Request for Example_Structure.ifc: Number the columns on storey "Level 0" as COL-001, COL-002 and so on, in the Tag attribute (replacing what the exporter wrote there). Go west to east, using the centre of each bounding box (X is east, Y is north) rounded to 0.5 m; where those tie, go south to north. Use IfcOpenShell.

First a look at what the model holds.

```python
import ifcopenshell
import ifcopenshell.util.element
import ifcopenshell.util.placement

model = ifcopenshell.open("Example_Structure.ifc")
print(model.schema)
storey = next(s for s in model.by_type("IfcBuildingStorey") if s.Name == "Level 0")
columns = [e for e in ifcopenshell.util.element.get_decomposition(storey) if e.is_a("IfcColumn")]
for e in sorted(columns, key=lambda e: e.id()):
    origin = ifcopenshell.util.placement.get_local_placement(e.ObjectPlacement)[:3, 3]
    print(e.id(), e.Tag, e.Name, origin.round(2) + 0.0, sep=" | ")
```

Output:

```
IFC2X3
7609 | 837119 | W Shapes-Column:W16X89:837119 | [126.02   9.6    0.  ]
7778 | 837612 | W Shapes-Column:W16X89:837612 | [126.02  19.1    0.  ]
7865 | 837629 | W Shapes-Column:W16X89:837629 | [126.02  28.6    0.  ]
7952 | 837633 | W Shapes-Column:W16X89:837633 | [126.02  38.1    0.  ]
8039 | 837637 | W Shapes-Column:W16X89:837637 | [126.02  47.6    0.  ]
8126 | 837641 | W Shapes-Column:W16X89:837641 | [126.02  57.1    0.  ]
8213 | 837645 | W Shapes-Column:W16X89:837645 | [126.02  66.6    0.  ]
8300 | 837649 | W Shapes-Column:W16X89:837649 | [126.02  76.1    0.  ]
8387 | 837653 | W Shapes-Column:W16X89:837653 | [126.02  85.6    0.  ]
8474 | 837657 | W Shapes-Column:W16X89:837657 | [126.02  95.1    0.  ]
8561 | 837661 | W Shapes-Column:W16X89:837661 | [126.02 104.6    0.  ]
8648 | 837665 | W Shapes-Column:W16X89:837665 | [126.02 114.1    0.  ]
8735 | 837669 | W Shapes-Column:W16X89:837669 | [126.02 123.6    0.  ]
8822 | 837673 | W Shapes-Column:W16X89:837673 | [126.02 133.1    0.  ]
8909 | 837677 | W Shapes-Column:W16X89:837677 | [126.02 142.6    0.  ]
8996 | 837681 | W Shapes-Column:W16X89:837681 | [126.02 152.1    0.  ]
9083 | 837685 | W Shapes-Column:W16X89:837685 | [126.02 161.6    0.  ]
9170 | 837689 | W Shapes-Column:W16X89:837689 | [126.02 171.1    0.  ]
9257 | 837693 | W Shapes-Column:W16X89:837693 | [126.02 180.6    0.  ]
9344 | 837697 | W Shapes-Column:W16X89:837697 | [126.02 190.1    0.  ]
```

```python
import ifcopenshell
import ifcopenshell.geom
import ifcopenshell.util.element
import ifcopenshell.util.shape

model = ifcopenshell.open("Example_Structure.ifc")
settings = ifcopenshell.geom.settings()
settings.set("use-world-coords", True)


def centre(element):
    shape = ifcopenshell.geom.create_shape(settings, element)
    return ifcopenshell.util.shape.get_bbox_centroid(shape.geometry)


storey = next(s for s in model.by_type("IfcBuildingStorey") if s.Name == "Level 0")
columns = [e for e in ifcopenshell.util.element.get_decomposition(storey) if e.is_a("IfcColumn")]

# Insertion points can sit at a corner or the storey origin, so sort by the geometry (in metres).
centres = {e: centre(e) for e in columns}
columns.sort(key=lambda e: (round(centres[e][0] / 0.5), centres[e][1]))

for i, e in enumerate(columns, start=1):
    number = f"COL-0{i:02d}"
    e.Tag = number
    print(e.id(), number)

model.write("Example_Structure_updated.ifc")
```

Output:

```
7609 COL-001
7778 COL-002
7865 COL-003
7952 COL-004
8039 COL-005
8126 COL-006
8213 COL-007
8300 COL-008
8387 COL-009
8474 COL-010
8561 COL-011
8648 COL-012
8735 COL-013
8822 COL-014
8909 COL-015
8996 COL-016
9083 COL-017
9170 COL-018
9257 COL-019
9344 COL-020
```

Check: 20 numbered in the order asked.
